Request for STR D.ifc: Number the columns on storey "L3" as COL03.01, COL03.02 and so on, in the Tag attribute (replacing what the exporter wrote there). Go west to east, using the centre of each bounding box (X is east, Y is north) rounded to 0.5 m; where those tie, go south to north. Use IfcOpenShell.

First a look at what the model holds.

```python
import ifcopenshell
import ifcopenshell.util.element
import ifcopenshell.util.placement

model = ifcopenshell.open("STR D.ifc")
print(model.schema)
storey = next(s for s in model.by_type("IfcBuildingStorey") if s.Name == "L3")
columns = [e for e in ifcopenshell.util.element.get_decomposition(storey) if e.is_a("IfcColumn")]
for e in sorted(columns, key=lambda e: e.id()):
    origin = ifcopenshell.util.placement.get_local_placement(e.ObjectPlacement)[:3, 3]
    print(e.id(), e.Tag, e.Name, origin.round(2) + 0.0, sep=" | ")
```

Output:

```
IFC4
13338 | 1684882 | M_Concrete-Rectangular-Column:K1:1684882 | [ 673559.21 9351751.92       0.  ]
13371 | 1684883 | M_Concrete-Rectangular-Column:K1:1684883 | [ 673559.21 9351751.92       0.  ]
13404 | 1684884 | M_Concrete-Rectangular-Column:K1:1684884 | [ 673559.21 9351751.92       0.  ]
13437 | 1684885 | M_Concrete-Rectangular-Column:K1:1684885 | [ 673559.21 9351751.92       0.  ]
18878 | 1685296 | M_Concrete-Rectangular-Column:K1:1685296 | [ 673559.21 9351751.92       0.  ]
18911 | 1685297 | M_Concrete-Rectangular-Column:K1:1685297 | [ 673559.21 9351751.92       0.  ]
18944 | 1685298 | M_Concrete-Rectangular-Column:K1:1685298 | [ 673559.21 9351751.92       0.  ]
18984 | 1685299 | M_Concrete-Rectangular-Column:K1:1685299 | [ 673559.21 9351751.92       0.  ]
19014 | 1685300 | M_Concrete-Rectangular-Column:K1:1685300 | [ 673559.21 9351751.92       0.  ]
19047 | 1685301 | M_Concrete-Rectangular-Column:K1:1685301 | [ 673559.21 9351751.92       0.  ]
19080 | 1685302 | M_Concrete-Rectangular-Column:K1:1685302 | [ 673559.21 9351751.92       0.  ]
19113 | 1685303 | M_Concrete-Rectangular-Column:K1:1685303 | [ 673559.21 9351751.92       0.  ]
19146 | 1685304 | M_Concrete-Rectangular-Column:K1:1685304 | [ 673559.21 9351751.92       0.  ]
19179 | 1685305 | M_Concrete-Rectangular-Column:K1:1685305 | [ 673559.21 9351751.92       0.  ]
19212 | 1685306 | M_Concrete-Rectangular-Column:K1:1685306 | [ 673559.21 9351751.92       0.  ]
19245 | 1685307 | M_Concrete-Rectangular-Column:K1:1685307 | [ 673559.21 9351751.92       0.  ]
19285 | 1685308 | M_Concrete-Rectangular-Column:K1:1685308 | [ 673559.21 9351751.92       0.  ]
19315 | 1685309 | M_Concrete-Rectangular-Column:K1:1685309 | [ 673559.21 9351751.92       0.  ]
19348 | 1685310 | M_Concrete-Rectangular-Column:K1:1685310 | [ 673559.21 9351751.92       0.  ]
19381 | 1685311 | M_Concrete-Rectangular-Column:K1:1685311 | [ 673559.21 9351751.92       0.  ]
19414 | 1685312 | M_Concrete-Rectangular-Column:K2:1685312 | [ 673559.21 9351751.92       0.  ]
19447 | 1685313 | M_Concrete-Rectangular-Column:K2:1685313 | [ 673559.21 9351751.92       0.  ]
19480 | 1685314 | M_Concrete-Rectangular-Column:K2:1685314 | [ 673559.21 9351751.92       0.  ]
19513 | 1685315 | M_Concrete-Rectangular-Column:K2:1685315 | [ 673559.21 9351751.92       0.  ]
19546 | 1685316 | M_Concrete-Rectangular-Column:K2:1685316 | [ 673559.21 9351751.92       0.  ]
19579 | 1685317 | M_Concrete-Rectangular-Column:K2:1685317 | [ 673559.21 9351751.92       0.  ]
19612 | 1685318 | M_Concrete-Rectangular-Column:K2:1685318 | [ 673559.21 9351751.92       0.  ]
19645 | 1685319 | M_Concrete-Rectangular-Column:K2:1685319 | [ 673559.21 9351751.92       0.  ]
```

```python
import ifcopenshell
import ifcopenshell.geom
import ifcopenshell.util.element
import ifcopenshell.util.shape

model = ifcopenshell.open("STR D.ifc")
settings = ifcopenshell.geom.settings()
settings.set("use-world-coords", True)


def centre(element):
    shape = ifcopenshell.geom.create_shape(settings, element)
    return ifcopenshell.util.shape.get_bbox_centroid(shape.geometry)


storey = next(s for s in model.by_type("IfcBuildingStorey") if s.Name == "L3")
columns = [e for e in ifcopenshell.util.element.get_decomposition(storey) if e.is_a("IfcColumn")]

# Insertion points can sit at a corner or the storey origin, so sort by the geometry (in metres).
centres = {e: centre(e) for e in columns}
columns.sort(key=lambda e: (round(centres[e][0] / 0.5), centres[e][1]))

for i, e in enumerate(columns, start=1):
    number = f"COL03.{i:02d}"
    e.Tag = number
    print(e.id(), number)

model.write("STR D_updated.ifc")
```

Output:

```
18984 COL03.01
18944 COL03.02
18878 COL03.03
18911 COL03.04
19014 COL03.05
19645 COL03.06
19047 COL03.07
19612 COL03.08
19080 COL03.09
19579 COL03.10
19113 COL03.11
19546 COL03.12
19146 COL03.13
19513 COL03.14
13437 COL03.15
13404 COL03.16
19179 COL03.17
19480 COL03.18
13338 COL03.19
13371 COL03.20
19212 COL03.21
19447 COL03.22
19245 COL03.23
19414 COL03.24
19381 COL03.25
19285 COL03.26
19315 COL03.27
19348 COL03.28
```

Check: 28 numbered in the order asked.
